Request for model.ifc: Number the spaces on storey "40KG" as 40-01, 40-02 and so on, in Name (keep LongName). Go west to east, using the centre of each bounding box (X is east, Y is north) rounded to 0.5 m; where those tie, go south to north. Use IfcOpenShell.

First a look at what the model holds.

```python
import ifcopenshell
import ifcopenshell.util.element
import ifcopenshell.util.placement

model = ifcopenshell.open("model.ifc")
print(model.schema)
storey = next(s for s in model.by_type("IfcBuildingStorey") if s.Name == "40KG")
spaces = [e for e in ifcopenshell.util.element.get_decomposition(storey) if e.is_a("IfcSpace")]
for e in sorted(spaces, key=lambda e: e.id()):
    origin = ifcopenshell.util.placement.get_local_placement(e.ObjectPlacement)[:3, 3]
    print(e.id(), e.Name, e.LongName, origin.round(2) + 0.0, sep=" | ")
```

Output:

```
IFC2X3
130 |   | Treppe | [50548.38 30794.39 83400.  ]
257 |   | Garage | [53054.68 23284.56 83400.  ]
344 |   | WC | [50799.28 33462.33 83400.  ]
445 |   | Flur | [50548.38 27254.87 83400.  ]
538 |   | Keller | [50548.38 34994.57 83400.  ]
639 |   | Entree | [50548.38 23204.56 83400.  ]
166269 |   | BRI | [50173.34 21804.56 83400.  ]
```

```python
import ifcopenshell
import ifcopenshell.geom
import ifcopenshell.util.element
import ifcopenshell.util.shape

model = ifcopenshell.open("model.ifc")
settings = ifcopenshell.geom.settings()
settings.set("use-world-coords", True)


def centre(element):
    shape = ifcopenshell.geom.create_shape(settings, element)
    return ifcopenshell.util.shape.get_bbox_centroid(shape.geometry)


storey = next(s for s in model.by_type("IfcBuildingStorey") if s.Name == "40KG")
spaces = [e for e in ifcopenshell.util.element.get_decomposition(storey) if e.is_a("IfcSpace")]

# Insertion points can sit at a corner or the storey origin, so sort by the geometry (in metres).
centres = {e: centre(e) for e in spaces}
spaces.sort(key=lambda e: (round(centres[e][0] / 0.5), centres[e][1]))

for i, e in enumerate(spaces, start=1):
    number = f"40-{i:02d}"
    e.Name = number
    print(e.id(), number)

model.write("model_v2.ifc")
```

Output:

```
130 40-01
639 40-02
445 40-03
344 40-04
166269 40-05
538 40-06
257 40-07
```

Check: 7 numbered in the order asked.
